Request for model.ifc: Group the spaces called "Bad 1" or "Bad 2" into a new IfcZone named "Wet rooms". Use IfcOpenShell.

First a look at what the model holds.

```python
import ifcopenshell

model = ifcopenshell.open("model.ifc")
print(model.schema)
seen = {}
for space in model.by_type("IfcSpace"):
    seen[space.LongName] = seen.get(space.LongName, 0) + 1
for name, count in sorted(seen.items(), key=str):
    print(count, "x", name)
print("zones:", [z.Name for z in model.by_type("IfcZone")][:20])
```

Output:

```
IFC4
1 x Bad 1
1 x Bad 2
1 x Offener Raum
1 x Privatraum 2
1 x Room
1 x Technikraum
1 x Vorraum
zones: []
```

```python
import ifcopenshell
import ifcopenshell.api.group
import ifcopenshell.api.root

model = ifcopenshell.open("model.ifc")

names = {"Bad 1", "Bad 2"}
spaces = [s for s in model.by_type("IfcSpace") if s.LongName in names]

zone = ifcopenshell.api.root.create_entity(model, ifc_class="IfcZone", name="Wet rooms")
ifcopenshell.api.group.assign_group(model, products=spaces, group=zone)
print(len(spaces), "spaces in", zone.Name)

model.write("model_updated.ifc")
```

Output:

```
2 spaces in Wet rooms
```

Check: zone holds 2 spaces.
